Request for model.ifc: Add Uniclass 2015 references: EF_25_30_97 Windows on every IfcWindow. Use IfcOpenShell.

First a look at what the model holds.

```python
import ifcopenshell

model = ifcopenshell.open("model.ifc")
print(model.schema)
print("classifications:", [c.Name for c in model.by_type("IfcClassification")])
for ifc_class in ("IfcDoor", "IfcRoof", "IfcStair", "IfcWall", "IfcWindow"):
    print(ifc_class, len(model.by_type(ifc_class)))
```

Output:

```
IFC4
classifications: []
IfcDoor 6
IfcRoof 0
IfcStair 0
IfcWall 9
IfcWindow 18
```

```python
import ifcopenshell
import ifcopenshell.api.classification

model = ifcopenshell.open("model.ifc")

system = ifcopenshell.api.classification.add_classification(model, classification="Uniclass 2015")

codes = {
    "IfcWindow": ("EF_25_30_97", "Windows"),
}
for ifc_class, (code, name) in codes.items():
    products = model.by_type(ifc_class)
    ifcopenshell.api.classification.add_reference(
        model, products=products, classification=system, identification=code, name=name
    )
    print(code, len(products))

model.write("model_edited.ifc")
```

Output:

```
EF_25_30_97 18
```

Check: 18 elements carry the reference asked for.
